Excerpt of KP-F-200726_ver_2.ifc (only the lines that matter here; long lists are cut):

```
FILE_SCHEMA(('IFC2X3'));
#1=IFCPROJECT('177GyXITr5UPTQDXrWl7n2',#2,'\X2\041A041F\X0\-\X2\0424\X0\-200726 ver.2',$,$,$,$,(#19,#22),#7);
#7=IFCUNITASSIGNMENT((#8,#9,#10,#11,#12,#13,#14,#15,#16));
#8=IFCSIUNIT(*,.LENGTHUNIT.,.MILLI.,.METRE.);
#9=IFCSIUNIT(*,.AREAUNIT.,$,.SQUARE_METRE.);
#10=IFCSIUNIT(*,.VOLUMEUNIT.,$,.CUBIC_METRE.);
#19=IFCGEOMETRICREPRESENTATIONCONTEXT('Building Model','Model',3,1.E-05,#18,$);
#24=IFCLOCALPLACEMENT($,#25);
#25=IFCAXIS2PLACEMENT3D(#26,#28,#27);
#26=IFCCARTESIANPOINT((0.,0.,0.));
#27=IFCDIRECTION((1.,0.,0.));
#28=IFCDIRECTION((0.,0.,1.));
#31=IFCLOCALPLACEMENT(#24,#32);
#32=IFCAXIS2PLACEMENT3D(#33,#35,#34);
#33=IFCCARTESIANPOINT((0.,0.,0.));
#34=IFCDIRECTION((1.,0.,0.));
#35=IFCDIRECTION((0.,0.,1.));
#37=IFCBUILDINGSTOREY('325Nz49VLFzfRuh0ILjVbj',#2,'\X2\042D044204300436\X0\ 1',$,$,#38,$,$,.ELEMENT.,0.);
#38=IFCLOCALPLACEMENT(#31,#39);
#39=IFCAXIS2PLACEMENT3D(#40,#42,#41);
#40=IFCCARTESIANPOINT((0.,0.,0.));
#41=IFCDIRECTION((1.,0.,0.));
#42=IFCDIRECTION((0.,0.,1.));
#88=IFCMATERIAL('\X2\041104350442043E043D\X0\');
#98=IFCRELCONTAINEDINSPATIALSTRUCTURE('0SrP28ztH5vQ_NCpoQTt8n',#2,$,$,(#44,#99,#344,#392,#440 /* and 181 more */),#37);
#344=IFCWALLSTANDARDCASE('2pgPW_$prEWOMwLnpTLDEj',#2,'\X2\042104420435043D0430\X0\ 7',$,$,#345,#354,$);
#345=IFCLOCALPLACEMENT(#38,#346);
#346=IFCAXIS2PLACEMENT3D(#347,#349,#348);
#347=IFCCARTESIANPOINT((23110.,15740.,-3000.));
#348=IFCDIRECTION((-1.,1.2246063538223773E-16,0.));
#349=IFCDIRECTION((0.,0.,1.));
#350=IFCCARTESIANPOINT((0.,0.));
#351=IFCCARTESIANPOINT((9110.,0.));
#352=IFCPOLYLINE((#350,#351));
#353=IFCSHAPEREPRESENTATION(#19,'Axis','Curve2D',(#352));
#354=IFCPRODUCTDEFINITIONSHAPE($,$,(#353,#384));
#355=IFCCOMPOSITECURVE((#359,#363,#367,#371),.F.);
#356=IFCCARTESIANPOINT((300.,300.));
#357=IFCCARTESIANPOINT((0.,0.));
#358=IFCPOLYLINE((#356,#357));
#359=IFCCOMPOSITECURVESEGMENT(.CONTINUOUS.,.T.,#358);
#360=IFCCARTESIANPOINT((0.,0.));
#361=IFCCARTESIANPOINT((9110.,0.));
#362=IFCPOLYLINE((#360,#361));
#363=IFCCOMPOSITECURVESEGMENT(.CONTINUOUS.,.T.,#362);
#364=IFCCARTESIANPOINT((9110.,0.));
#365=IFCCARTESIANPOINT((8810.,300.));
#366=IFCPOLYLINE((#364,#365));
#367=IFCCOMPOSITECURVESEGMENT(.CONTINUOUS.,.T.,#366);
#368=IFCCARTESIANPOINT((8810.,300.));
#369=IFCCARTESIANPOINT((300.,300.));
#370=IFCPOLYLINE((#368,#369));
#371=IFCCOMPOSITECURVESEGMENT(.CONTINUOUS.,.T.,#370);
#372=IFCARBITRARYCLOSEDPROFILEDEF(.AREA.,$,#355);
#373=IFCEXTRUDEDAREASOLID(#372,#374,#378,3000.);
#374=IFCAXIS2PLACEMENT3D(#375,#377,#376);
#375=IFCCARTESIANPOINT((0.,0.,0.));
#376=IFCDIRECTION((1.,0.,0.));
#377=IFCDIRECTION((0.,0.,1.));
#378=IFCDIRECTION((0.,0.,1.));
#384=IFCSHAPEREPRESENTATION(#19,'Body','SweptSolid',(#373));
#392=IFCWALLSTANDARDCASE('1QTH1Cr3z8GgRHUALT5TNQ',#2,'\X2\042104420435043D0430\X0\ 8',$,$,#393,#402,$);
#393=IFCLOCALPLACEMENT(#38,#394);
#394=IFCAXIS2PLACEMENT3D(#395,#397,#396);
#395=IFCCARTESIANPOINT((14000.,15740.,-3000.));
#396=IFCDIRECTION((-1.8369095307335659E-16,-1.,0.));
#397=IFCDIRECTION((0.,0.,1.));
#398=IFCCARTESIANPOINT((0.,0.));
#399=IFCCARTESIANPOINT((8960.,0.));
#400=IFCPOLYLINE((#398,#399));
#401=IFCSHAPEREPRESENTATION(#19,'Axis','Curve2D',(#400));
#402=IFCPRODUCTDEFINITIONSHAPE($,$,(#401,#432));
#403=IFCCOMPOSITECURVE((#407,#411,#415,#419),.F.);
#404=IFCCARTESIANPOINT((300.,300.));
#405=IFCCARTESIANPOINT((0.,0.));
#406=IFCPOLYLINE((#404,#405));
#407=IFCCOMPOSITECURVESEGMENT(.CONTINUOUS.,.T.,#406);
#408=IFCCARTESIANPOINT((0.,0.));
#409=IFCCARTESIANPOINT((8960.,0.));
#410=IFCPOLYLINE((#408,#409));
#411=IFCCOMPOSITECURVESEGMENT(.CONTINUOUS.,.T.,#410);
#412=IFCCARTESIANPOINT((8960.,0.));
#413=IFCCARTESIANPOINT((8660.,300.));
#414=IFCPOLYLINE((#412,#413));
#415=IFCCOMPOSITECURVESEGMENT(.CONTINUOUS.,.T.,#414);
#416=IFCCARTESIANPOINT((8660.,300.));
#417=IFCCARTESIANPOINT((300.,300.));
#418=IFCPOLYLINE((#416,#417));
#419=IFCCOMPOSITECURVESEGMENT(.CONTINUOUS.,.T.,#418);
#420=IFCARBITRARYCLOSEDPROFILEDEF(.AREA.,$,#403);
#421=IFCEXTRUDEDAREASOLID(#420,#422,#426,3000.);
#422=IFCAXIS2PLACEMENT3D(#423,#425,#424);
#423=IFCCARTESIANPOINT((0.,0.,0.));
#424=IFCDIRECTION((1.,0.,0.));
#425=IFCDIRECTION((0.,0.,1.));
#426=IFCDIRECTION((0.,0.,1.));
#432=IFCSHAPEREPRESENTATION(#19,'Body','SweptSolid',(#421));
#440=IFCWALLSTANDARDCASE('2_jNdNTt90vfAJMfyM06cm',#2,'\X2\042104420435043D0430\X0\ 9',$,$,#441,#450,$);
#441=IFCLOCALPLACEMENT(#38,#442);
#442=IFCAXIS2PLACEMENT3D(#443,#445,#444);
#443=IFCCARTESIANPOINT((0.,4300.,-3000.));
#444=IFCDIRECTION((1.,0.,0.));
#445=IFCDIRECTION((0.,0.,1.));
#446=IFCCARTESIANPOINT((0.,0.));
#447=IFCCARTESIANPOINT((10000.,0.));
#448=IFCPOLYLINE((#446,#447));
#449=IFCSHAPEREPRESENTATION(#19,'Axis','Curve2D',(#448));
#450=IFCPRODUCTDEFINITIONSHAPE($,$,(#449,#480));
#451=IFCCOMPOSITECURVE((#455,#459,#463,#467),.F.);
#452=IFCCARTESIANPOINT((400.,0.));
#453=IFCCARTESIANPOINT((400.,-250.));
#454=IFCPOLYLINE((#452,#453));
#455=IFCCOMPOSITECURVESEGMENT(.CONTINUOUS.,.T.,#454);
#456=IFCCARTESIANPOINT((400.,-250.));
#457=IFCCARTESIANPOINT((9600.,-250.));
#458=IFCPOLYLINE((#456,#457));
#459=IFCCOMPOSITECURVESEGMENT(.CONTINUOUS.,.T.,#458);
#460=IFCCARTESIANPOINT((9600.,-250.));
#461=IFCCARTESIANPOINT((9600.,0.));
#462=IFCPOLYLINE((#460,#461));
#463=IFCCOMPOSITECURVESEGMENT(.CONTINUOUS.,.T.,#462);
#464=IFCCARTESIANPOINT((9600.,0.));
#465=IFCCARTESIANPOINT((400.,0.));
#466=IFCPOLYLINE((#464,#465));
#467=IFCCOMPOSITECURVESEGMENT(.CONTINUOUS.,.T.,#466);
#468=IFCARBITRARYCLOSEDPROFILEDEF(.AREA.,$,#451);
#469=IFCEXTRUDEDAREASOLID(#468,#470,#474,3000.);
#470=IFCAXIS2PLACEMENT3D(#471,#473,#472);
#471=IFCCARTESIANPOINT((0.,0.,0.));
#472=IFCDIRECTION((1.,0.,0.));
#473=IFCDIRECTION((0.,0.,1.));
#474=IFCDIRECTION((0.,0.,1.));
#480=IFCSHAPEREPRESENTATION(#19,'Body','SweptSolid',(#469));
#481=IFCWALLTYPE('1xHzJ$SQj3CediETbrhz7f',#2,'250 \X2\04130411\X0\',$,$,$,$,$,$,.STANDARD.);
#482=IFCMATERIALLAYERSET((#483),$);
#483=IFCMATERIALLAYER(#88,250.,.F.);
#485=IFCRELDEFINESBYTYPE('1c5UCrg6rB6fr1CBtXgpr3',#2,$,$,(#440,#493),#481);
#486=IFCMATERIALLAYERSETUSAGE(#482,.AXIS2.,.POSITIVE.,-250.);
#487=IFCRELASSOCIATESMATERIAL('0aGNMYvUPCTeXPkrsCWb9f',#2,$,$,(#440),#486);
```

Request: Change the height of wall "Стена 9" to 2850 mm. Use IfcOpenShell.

```python
import ifcopenshell
import ifcopenshell.geom
import ifcopenshell.util.shape

model = ifcopenshell.open("KP-F-200726_ver_2.ifc")
settings = ifcopenshell.geom.settings()


def volume(element):
    """Net volume in cubic metres, openings subtracted."""
    shape = ifcopenshell.geom.create_shape(settings, element)
    return ifcopenshell.util.shape.get_volume(shape.geometry)


wall = model.by_id(440)
before = volume(wall)

body = next(r for r in wall.Representation.Representations if r.RepresentationIdentifier == "Body")
solid = body.Items[0]
old_height = solid.Depth
solid.Depth = 2850.0
after = volume(wall)

print(f"height {old_height:g} -> {solid.Depth:g}, volume {before:.3f} -> {after:.3f} m3")

model.write("KP-F-200726_ver_2_updated.ifc")
```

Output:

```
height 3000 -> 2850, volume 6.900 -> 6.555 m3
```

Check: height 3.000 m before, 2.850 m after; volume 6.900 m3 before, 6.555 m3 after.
